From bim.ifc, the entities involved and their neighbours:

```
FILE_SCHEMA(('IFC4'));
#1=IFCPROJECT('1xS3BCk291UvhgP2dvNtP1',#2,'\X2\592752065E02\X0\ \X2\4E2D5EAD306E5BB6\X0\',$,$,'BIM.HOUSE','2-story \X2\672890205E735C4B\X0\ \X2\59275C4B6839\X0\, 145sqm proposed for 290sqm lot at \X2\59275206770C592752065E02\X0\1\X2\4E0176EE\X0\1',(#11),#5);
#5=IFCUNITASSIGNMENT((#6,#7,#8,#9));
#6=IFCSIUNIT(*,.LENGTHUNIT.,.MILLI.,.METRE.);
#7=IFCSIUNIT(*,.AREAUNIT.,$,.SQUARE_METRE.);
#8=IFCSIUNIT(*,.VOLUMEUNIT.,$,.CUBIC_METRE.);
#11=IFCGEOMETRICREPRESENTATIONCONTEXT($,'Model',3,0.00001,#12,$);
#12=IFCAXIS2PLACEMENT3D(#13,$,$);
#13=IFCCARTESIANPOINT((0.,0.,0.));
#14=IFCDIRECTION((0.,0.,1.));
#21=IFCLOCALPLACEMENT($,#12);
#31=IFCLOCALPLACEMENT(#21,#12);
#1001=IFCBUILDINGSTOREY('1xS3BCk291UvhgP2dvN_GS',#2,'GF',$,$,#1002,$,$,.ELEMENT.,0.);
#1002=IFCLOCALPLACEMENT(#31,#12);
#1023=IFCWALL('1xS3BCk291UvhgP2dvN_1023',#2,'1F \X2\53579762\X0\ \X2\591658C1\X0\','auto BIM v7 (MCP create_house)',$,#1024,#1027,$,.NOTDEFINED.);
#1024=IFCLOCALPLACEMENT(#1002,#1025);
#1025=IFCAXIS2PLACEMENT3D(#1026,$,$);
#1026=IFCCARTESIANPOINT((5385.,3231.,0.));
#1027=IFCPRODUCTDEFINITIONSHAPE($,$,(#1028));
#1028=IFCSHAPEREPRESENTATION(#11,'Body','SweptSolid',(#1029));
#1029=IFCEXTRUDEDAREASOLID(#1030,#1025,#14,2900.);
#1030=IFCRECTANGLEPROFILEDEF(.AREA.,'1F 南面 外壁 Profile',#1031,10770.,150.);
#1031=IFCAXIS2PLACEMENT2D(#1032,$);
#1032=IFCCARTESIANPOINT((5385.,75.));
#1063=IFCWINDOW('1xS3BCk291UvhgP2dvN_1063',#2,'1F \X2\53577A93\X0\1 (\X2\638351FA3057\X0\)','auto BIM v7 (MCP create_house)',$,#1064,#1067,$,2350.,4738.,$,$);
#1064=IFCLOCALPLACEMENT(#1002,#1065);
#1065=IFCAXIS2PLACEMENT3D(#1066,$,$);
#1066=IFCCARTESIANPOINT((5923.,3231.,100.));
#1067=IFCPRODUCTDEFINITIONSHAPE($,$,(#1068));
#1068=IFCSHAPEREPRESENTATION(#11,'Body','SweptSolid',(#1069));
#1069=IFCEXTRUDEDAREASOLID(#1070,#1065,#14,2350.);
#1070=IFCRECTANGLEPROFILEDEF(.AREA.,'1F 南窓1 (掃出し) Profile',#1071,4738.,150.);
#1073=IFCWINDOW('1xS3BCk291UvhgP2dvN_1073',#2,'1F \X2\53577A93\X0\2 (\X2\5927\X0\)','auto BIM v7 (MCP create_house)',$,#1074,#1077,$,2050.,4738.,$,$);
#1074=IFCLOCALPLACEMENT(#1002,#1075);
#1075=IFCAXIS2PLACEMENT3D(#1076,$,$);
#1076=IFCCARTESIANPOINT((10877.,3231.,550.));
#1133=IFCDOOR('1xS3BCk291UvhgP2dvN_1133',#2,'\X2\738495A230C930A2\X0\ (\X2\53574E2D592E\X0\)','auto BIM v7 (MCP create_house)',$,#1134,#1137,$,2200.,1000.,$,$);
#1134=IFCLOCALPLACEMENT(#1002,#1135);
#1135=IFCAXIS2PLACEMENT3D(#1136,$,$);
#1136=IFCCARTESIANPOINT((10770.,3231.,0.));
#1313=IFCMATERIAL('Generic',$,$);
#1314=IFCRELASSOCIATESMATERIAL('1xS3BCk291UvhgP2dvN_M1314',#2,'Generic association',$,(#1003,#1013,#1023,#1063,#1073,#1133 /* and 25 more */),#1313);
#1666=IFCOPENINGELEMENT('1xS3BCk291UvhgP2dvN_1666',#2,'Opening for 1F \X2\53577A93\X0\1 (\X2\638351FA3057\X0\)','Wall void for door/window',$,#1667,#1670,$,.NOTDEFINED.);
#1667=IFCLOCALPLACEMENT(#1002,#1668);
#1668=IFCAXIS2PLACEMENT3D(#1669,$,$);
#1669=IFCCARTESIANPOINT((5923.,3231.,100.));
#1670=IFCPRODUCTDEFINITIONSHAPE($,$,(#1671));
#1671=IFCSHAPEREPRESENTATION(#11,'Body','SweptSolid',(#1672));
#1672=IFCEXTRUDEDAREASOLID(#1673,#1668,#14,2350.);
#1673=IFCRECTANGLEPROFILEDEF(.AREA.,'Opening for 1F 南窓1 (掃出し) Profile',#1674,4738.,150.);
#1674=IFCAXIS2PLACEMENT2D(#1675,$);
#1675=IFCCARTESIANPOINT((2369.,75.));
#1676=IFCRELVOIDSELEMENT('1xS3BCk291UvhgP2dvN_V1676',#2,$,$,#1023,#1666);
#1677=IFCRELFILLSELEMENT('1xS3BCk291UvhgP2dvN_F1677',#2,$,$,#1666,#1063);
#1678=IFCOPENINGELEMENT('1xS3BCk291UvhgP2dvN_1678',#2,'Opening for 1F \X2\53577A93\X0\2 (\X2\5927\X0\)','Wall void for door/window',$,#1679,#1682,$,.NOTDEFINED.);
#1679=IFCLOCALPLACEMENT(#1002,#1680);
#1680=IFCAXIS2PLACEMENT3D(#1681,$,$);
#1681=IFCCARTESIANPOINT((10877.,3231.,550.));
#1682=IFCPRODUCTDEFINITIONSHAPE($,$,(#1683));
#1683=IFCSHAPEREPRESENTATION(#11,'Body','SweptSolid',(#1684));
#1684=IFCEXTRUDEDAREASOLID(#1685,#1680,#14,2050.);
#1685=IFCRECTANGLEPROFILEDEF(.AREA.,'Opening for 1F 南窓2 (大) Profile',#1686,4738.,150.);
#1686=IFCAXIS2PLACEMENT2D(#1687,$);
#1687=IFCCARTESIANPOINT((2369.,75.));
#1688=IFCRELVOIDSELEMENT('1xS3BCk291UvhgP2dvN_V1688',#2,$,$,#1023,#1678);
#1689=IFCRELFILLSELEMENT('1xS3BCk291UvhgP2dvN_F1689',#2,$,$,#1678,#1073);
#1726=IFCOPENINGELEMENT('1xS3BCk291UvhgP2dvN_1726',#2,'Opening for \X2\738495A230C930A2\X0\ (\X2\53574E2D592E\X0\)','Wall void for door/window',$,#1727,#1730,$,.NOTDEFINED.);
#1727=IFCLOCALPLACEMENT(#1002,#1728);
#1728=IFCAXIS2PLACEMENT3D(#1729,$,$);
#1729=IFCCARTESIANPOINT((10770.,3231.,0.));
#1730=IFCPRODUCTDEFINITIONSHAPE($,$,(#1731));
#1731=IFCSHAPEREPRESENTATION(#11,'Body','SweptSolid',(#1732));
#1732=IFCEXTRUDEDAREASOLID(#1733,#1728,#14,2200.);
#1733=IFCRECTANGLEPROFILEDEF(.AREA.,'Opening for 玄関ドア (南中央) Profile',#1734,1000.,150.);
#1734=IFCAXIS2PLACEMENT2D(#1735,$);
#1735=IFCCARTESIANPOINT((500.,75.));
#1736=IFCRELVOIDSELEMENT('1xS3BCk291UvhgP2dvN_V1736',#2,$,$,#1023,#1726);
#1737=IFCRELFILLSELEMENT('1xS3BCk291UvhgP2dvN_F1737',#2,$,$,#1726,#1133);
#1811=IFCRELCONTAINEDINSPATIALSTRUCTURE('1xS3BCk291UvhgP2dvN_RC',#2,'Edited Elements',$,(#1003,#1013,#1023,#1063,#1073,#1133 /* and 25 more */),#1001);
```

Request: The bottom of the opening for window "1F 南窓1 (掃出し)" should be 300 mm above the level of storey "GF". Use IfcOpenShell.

```python
import numpy as np
import ifcopenshell
import ifcopenshell.api.geometry
import ifcopenshell.geom
import ifcopenshell.util.element
import ifcopenshell.util.placement
import ifcopenshell.util.shape
import ifcopenshell.util.unit

model = ifcopenshell.open("bim.ifc")
unit_scale = ifcopenshell.util.unit.calculate_unit_scale(model)

window = model.by_id(1063)
opening = window.FillsVoids[0].RelatingOpeningElement
storey = ifcopenshell.util.element.get_container(window, ifc_class="IfcBuildingStorey")
level = ifcopenshell.util.placement.get_local_placement(storey.ObjectPlacement)[2, 3]

# The opening's origin need not be at the sill, so measure its lowest point.
shape = ifcopenshell.geom.create_shape(ifcopenshell.geom.settings(), opening)
bottom = ifcopenshell.util.shape.get_shape_bottom_elevation(shape, shape.geometry) / unit_scale
dz = level + 0.3 / unit_scale - bottom

shift = np.array([0.0, 0.0, dz])
# The window is not placed relative to its opening, so move both.
for product in (opening, window):
    matrix = ifcopenshell.util.placement.get_local_placement(product.ObjectPlacement)
    matrix[:3, 3] += shift
    ifcopenshell.api.geometry.edit_object_placement(model, product=product, matrix=matrix, is_si=False)

print(f"moved by {dz * unit_scale:+.3f} m")

model.write("bim-out.ifc")
```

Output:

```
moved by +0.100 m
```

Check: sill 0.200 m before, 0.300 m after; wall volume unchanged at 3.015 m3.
